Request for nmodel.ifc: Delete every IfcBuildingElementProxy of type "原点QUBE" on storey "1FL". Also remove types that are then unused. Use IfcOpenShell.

First a look at what the model holds.

```python
import ifcopenshell
import ifcopenshell.util.element

model = ifcopenshell.open("nmodel.ifc")
print(model.schema)
storey = next(s for s in model.by_type("IfcBuildingStorey") if s.Name == "1FL")
proxies = [e for e in ifcopenshell.util.element.get_decomposition(storey) if e.is_a("IfcBuildingElementProxy")]
seen = {}
for e in proxies:
    element_type = ifcopenshell.util.element.get_type(e)
    name = element_type.Name if element_type not in (None, e) else None
    seen[name] = seen.get(name, 0) + 1
for name, count in sorted(seen.items(), key=str):
    print(count, "x", name)
```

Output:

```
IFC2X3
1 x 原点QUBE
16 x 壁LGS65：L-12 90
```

```python
import ifcopenshell
import ifcopenshell.api.root
import ifcopenshell.util.element

model = ifcopenshell.open("nmodel.ifc")

storey = next(s for s in model.by_type("IfcBuildingStorey") if s.Name == "1FL")
proxies = [e for e in ifcopenshell.util.element.get_decomposition(storey) if e.is_a("IfcBuildingElementProxy")]
targets = [e for e in proxies if (t := ifcopenshell.util.element.get_type(e)) not in (None, e) and t.Name == "原点QUBE"]
types = {ifcopenshell.util.element.get_type(e) for e in targets} - {None, *targets}

for e in targets:
    ifcopenshell.api.root.remove_product(model, product=e)
print(len(targets), "removed")

unused = [t for t in types if not ifcopenshell.util.element.get_types(t)]
for t in unused:
    ifcopenshell.api.root.remove_product(model, product=t)
print(len(unused), "unused types removed")

model.write("nmodel_rev.ifc")
```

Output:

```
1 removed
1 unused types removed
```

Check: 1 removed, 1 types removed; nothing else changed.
